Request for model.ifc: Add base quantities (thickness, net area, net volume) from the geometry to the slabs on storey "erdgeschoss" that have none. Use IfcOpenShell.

First a look at what the model holds.

```python
import ifcopenshell
import ifcopenshell.util.element
import ifcopenshell.util.unit

model = ifcopenshell.open("model.ifc")
print(model.schema)
for unit_type in ("LENGTHUNIT", "AREAUNIT", "VOLUMEUNIT"):
    print(unit_type, ifcopenshell.util.unit.calculate_unit_scale(model, unit_type))
storey = next(s for s in model.by_type("IfcBuildingStorey") if s.Name == "erdgeschoss")
slabs = [e for e in ifcopenshell.util.element.get_decomposition(storey) if e.is_a("IfcSlab")]
for e in sorted(slabs, key=lambda e: e.id()):
    print(e.id(), e.is_a(), e.Name, list(ifcopenshell.util.element.get_psets(e, qtos_only=True)), sep=" | ")
```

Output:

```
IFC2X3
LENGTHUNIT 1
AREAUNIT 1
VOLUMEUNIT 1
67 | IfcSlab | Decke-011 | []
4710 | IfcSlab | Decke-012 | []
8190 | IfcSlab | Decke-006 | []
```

```python
import ifcopenshell
import ifcopenshell.api.pset
import ifcopenshell.geom
import ifcopenshell.util.element
import ifcopenshell.util.shape
import ifcopenshell.util.unit

model = ifcopenshell.open("model.ifc")
unit_scale = ifcopenshell.util.unit.calculate_unit_scale(model)
area_scale = ifcopenshell.util.unit.calculate_unit_scale(model, "AREAUNIT")
volume_scale = ifcopenshell.util.unit.calculate_unit_scale(model, "VOLUMEUNIT")
settings = ifcopenshell.geom.settings()

storey = next(s for s in model.by_type("IfcBuildingStorey") if s.Name == "erdgeschoss")
slabs = [e for e in ifcopenshell.util.element.get_decomposition(storey) if e.is_a("IfcSlab")]

for e in sorted(slabs, key=lambda e: e.id()):
    if ifcopenshell.util.element.get_psets(e, qtos_only=True, should_inherit=False):
        continue
    # Geometry comes back in metres, in the element's own axes.
    shape = ifcopenshell.geom.create_shape(settings, e)
    values = {
        "Width": ifcopenshell.util.shape.get_z(shape.geometry) / unit_scale,
        "NetArea": ifcopenshell.util.shape.get_footprint_area(shape.geometry) / area_scale,
        "NetVolume": ifcopenshell.util.shape.get_volume(shape.geometry) / volume_scale,
    }
    qto = ifcopenshell.api.pset.add_qto(model, product=e, name="BaseQuantities")
    ifcopenshell.api.pset.edit_qto(model, qto=qto, properties=values)
    print(e.id(), {k: round(v, 3) for k, v in values.items()})

model.write("model_edited.ifc")
```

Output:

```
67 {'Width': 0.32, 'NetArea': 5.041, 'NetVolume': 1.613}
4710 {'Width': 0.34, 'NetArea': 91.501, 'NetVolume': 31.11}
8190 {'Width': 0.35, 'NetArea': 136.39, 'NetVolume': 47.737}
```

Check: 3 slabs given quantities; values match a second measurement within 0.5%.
